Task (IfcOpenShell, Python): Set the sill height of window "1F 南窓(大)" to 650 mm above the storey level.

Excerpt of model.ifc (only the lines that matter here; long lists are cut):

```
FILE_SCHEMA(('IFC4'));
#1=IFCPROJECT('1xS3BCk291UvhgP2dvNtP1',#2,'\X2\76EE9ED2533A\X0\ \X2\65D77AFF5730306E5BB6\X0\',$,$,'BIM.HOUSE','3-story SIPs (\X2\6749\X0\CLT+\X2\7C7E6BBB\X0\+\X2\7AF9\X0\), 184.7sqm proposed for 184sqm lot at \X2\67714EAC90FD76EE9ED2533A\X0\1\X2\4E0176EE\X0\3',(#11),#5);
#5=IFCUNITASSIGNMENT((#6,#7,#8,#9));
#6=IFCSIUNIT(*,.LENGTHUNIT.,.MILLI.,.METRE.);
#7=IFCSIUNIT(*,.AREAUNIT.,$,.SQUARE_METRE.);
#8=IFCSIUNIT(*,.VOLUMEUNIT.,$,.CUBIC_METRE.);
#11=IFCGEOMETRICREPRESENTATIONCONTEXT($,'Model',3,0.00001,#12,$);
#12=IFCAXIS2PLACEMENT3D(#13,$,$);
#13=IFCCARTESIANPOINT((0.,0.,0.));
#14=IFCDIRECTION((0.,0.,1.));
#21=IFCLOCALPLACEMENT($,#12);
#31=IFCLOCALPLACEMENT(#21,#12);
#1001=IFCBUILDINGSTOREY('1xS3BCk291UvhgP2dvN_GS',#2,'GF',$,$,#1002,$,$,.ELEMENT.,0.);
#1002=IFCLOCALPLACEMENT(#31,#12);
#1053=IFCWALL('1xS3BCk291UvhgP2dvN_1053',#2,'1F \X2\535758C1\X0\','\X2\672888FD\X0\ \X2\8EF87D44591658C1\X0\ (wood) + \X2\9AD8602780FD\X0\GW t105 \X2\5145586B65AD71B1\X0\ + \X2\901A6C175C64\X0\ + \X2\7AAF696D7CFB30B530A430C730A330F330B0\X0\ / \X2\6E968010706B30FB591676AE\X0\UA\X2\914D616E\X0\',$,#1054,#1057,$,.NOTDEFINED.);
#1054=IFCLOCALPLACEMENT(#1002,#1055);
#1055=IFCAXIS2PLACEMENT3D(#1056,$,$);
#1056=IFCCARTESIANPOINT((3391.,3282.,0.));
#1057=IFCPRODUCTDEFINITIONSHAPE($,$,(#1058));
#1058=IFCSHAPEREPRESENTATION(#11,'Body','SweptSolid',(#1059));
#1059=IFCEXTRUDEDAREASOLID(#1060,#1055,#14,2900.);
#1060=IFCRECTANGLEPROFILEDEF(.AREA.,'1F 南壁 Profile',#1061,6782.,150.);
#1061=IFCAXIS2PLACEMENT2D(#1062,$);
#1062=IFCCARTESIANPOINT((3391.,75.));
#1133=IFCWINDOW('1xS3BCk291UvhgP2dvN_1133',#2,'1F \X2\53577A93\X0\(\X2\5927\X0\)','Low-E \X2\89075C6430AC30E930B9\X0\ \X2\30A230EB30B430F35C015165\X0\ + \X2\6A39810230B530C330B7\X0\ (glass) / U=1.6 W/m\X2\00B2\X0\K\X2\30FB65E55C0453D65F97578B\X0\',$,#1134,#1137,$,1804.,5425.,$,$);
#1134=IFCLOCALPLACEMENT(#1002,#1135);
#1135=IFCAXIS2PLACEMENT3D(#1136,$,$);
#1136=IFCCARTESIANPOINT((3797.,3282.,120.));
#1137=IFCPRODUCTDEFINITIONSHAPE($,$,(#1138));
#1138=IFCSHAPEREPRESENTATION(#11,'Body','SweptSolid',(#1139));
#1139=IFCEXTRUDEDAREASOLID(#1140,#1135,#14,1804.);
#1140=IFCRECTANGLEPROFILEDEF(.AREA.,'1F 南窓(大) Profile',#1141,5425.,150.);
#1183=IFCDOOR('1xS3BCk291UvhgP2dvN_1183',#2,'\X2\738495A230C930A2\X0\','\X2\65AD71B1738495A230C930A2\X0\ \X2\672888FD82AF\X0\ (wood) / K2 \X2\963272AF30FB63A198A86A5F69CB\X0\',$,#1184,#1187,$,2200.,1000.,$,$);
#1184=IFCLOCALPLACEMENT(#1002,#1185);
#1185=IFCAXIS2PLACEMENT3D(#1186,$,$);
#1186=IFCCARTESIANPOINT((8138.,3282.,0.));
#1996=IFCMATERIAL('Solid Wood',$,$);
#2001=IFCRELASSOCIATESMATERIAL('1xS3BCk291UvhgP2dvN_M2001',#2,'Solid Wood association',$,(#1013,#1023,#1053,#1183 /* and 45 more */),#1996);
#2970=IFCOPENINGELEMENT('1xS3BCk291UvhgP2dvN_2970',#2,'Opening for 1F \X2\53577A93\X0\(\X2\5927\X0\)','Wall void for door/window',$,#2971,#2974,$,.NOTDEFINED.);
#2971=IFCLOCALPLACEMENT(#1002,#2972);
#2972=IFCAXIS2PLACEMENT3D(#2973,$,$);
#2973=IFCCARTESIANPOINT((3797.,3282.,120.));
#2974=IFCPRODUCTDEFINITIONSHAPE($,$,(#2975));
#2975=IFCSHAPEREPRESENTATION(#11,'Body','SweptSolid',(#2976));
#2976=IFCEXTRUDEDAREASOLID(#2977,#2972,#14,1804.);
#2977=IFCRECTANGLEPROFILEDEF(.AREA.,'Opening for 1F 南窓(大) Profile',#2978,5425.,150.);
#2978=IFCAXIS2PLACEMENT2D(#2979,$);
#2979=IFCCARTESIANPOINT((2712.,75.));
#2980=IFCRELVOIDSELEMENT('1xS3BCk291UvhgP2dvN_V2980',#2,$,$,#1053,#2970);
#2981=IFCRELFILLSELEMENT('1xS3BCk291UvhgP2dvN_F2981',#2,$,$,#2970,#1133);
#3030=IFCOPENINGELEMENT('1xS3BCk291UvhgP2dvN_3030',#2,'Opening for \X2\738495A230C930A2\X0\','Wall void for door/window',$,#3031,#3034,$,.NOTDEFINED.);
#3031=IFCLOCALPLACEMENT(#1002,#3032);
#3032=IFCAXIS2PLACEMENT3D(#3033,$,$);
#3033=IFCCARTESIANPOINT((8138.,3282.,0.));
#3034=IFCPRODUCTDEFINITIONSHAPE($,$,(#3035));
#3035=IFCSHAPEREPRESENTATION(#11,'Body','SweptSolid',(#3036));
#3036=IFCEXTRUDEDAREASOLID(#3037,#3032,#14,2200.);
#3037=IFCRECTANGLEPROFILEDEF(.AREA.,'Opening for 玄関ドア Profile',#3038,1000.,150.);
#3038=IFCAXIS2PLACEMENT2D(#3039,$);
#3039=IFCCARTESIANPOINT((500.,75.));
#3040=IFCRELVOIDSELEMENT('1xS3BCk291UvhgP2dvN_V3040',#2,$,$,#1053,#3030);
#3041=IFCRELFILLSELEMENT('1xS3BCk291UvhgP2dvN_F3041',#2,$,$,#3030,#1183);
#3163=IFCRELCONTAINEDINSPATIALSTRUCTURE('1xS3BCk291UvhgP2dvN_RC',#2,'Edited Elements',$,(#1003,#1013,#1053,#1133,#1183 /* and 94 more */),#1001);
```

```python
import numpy as np
import ifcopenshell
import ifcopenshell.api.geometry
import ifcopenshell.geom
import ifcopenshell.util.element
import ifcopenshell.util.placement
import ifcopenshell.util.shape
import ifcopenshell.util.unit

model = ifcopenshell.open("model.ifc")
unit_scale = ifcopenshell.util.unit.calculate_unit_scale(model)

window = model.by_guid("1xS3BCk291UvhgP2dvN_1133")
opening = window.FillsVoids[0].RelatingOpeningElement
storey = ifcopenshell.util.element.get_container(window, ifc_class="IfcBuildingStorey")
level = ifcopenshell.util.placement.get_local_placement(storey.ObjectPlacement)[2, 3]

# The opening's origin need not be at the sill, so measure its lowest point.
shape = ifcopenshell.geom.create_shape(ifcopenshell.geom.settings(), opening)
bottom = ifcopenshell.util.shape.get_shape_bottom_elevation(shape, shape.geometry) / unit_scale
dz = level + 0.65 / unit_scale - bottom

shift = np.array([0.0, 0.0, dz])
# The window is not placed relative to its opening, so move both.
for product in (opening, window):
    matrix = ifcopenshell.util.placement.get_local_placement(product.ObjectPlacement)
    matrix[:3, 3] += shift
    ifcopenshell.api.geometry.edit_object_placement(model, product=product, matrix=matrix, is_si=False)

print(f"moved by {dz * unit_scale:+.3f} m")

model.write("model_rev.ifc")
```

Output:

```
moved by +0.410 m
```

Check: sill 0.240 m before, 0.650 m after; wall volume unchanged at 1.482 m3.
